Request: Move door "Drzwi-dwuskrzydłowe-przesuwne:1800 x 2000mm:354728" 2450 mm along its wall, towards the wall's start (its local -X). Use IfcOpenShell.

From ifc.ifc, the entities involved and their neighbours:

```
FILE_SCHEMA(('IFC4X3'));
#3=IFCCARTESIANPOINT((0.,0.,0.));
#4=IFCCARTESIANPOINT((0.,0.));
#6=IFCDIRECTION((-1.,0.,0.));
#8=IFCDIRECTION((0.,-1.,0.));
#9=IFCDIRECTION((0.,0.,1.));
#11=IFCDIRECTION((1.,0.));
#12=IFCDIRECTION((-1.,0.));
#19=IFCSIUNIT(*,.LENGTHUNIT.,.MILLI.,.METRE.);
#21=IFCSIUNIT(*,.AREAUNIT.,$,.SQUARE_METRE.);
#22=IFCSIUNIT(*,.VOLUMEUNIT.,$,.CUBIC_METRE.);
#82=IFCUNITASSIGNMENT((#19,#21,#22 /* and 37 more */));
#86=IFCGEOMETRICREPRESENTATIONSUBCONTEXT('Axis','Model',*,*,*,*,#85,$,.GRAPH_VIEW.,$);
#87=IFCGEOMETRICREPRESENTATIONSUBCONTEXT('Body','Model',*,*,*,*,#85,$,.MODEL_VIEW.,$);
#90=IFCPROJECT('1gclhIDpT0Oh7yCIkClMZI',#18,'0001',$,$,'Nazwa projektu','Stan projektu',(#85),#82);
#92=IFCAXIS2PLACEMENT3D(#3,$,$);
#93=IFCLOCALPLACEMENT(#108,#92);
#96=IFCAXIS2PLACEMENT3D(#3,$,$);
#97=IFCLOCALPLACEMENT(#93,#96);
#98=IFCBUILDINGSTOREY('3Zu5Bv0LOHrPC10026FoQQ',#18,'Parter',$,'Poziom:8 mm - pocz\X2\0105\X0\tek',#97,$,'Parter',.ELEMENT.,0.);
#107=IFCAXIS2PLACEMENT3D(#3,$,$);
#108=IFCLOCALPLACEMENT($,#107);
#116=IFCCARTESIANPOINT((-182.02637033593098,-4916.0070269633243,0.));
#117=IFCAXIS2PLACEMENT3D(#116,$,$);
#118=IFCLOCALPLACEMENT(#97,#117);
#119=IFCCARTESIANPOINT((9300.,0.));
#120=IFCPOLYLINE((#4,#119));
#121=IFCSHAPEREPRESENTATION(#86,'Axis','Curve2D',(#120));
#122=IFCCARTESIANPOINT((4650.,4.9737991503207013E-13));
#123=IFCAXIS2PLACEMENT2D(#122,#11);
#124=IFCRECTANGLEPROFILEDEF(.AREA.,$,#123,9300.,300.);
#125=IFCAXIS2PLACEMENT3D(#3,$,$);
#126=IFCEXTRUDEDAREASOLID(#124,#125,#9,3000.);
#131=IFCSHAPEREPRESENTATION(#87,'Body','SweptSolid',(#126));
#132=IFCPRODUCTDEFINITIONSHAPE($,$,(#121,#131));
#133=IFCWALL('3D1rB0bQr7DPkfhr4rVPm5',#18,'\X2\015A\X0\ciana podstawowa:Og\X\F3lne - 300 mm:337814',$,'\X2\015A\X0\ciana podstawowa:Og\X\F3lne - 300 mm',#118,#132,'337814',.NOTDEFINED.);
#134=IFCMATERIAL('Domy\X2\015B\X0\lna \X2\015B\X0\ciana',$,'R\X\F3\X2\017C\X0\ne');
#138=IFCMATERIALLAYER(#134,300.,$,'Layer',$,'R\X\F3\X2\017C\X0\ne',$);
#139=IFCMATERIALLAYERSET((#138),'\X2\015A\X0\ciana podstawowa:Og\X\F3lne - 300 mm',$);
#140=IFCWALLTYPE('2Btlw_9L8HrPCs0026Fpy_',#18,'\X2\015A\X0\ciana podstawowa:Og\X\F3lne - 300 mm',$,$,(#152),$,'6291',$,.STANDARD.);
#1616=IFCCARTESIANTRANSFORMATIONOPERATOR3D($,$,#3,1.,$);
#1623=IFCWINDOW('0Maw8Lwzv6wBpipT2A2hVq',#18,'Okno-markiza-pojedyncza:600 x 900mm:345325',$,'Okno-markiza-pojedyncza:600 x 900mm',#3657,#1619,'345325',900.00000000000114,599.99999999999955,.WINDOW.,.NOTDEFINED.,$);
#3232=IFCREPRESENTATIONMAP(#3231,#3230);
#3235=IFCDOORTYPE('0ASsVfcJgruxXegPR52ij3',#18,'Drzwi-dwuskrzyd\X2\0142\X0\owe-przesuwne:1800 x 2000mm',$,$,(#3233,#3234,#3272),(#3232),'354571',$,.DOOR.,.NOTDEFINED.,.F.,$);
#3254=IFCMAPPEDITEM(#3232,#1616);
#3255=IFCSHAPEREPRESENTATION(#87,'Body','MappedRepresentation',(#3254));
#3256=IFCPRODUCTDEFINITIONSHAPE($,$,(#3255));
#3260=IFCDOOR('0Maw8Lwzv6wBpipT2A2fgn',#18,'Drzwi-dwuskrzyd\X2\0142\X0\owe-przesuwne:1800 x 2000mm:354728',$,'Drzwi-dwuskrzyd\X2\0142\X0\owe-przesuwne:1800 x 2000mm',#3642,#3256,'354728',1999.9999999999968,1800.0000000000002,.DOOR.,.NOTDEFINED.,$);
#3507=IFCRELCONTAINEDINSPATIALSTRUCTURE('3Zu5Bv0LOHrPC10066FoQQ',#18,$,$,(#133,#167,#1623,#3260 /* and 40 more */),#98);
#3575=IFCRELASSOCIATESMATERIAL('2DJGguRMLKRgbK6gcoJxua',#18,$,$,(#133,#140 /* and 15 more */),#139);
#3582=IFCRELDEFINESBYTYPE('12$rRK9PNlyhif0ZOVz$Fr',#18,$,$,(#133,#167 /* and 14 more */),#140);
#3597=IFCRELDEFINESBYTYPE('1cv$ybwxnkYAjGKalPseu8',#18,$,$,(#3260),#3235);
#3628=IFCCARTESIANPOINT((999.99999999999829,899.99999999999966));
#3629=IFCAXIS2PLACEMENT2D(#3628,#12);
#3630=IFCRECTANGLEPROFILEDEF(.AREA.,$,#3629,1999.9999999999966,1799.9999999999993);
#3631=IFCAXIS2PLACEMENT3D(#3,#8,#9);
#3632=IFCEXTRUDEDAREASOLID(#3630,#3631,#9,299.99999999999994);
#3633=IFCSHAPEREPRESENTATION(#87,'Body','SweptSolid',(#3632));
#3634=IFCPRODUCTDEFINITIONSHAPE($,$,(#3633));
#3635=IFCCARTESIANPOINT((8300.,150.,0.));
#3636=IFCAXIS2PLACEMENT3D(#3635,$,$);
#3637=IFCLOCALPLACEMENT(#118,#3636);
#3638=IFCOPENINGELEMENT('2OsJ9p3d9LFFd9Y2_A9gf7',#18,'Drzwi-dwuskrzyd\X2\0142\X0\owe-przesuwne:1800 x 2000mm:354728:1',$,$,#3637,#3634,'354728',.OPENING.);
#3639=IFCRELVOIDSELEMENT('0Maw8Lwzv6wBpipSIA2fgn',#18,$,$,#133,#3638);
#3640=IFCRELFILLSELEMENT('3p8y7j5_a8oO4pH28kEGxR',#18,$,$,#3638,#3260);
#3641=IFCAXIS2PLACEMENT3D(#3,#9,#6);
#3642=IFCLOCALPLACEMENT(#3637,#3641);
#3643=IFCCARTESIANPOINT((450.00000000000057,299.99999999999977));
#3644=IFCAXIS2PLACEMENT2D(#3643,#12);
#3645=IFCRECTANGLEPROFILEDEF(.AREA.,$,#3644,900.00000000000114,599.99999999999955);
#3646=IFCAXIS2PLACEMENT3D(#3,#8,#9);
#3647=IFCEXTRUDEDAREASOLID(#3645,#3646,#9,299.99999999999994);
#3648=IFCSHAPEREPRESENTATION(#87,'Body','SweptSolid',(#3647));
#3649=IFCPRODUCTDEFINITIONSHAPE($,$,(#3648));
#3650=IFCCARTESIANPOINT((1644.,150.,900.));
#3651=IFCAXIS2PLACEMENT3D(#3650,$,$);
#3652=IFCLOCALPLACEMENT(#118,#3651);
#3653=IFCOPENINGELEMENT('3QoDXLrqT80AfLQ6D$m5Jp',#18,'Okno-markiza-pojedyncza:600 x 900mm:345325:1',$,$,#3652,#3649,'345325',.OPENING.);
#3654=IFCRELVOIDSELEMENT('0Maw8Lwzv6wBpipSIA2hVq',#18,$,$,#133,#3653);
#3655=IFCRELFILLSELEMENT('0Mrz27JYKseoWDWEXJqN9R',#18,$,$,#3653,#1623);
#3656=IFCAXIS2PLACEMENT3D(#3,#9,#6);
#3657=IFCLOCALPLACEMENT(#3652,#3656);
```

```python
import ifcopenshell
import ifcopenshell.api.geometry
import ifcopenshell.util.placement

model = ifcopenshell.open("ifc.ifc")

door = model.by_id(3260)
opening = door.FillsVoids[0].RelatingOpeningElement
wall = opening.VoidsElements[0].RelatingBuildingElement

wall_matrix = ifcopenshell.util.placement.get_local_placement(wall.ObjectPlacement)
shift = wall_matrix[:3, 0] * -2450.0
before = ifcopenshell.util.placement.get_local_placement(door.ObjectPlacement)[:3, 3].copy()

# The door is placed relative to its opening, so it follows when the opening moves.
matrix = ifcopenshell.util.placement.get_local_placement(opening.ObjectPlacement)
matrix[:3, 3] += shift
ifcopenshell.api.geometry.edit_object_placement(
    model, product=opening, matrix=matrix, is_si=False, should_transform_children=True
)

after = ifcopenshell.util.placement.get_local_placement(door.ObjectPlacement)[:3, 3]
print("door moved by", (after - before).round(3) + 0.0)

model.write("ifc_updated.ifc")
```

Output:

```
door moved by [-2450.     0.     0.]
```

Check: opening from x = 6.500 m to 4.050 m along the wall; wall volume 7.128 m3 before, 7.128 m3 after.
